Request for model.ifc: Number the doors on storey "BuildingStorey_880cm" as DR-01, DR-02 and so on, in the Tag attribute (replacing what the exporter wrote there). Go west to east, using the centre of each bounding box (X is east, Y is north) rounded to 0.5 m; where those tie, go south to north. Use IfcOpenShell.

First a look at what the model holds.

```python
import ifcopenshell
import ifcopenshell.util.element
import ifcopenshell.util.placement

model = ifcopenshell.open("model.ifc")
print(model.schema)
storey = next(s for s in model.by_type("IfcBuildingStorey") if s.Name == "BuildingStorey_880cm")
doors = [e for e in ifcopenshell.util.element.get_decomposition(storey) if e.is_a("IfcDoor")]
for e in sorted(doors, key=lambda e: e.id()):
    origin = ifcopenshell.util.placement.get_local_placement(e.ObjectPlacement)[:3, 3]
    print(e.id(), e.Tag, e.Name, origin.round(2) + 0.0, sep=" | ")
```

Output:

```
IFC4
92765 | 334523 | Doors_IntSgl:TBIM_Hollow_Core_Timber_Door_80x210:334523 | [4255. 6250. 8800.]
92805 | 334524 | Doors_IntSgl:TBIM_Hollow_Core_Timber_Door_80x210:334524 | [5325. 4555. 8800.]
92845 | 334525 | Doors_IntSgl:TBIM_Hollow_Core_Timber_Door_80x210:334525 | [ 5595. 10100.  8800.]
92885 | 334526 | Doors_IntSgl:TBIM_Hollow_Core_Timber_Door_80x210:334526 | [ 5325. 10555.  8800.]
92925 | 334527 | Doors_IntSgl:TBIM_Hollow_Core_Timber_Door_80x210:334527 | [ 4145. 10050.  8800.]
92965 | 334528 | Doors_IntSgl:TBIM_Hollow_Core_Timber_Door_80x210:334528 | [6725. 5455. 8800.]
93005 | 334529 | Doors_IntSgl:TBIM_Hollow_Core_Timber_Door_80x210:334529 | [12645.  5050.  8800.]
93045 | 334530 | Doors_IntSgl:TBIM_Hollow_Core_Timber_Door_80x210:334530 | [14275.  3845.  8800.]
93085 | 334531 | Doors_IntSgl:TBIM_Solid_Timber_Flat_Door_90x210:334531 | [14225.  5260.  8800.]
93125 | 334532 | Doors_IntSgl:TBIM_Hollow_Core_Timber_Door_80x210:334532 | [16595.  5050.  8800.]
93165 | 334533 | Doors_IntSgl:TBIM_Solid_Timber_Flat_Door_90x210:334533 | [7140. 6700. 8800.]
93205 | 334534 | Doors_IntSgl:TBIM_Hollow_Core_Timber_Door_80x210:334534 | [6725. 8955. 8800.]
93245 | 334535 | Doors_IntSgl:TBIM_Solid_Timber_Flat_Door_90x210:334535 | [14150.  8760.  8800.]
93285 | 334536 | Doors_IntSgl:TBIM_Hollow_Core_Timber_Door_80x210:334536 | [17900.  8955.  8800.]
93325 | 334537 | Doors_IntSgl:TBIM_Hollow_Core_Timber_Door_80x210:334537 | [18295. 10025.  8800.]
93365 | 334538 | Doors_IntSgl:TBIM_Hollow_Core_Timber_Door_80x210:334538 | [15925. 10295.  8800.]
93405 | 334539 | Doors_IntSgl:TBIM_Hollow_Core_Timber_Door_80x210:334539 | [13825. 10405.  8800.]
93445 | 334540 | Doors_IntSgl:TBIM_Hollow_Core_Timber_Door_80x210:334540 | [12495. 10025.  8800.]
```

```python
import ifcopenshell
import ifcopenshell.geom
import ifcopenshell.util.element
import ifcopenshell.util.shape

model = ifcopenshell.open("model.ifc")
settings = ifcopenshell.geom.settings()
settings.set("use-world-coords", True)


def centre(element):
    shape = ifcopenshell.geom.create_shape(settings, element)
    return ifcopenshell.util.shape.get_bbox_centroid(shape.geometry)


storey = next(s for s in model.by_type("IfcBuildingStorey") if s.Name == "BuildingStorey_880cm")
doors = [e for e in ifcopenshell.util.element.get_decomposition(storey) if e.is_a("IfcDoor")]

# Insertion points can sit at a corner or the storey origin, so sort by the geometry (in metres).
centres = {e: centre(e) for e in doors}
doors.sort(key=lambda e: (round(centres[e][0] / 0.5), centres[e][1]))

for i, e in enumerate(doors, start=1):
    number = f"DR-{i:02d}"
    e.Tag = number
    print(e.id(), number)

model.write("model_updated.ifc")
```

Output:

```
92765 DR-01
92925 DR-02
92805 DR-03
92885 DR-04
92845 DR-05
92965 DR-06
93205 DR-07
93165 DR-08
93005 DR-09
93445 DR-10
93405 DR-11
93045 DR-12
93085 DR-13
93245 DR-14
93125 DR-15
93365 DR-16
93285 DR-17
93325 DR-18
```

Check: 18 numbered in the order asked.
